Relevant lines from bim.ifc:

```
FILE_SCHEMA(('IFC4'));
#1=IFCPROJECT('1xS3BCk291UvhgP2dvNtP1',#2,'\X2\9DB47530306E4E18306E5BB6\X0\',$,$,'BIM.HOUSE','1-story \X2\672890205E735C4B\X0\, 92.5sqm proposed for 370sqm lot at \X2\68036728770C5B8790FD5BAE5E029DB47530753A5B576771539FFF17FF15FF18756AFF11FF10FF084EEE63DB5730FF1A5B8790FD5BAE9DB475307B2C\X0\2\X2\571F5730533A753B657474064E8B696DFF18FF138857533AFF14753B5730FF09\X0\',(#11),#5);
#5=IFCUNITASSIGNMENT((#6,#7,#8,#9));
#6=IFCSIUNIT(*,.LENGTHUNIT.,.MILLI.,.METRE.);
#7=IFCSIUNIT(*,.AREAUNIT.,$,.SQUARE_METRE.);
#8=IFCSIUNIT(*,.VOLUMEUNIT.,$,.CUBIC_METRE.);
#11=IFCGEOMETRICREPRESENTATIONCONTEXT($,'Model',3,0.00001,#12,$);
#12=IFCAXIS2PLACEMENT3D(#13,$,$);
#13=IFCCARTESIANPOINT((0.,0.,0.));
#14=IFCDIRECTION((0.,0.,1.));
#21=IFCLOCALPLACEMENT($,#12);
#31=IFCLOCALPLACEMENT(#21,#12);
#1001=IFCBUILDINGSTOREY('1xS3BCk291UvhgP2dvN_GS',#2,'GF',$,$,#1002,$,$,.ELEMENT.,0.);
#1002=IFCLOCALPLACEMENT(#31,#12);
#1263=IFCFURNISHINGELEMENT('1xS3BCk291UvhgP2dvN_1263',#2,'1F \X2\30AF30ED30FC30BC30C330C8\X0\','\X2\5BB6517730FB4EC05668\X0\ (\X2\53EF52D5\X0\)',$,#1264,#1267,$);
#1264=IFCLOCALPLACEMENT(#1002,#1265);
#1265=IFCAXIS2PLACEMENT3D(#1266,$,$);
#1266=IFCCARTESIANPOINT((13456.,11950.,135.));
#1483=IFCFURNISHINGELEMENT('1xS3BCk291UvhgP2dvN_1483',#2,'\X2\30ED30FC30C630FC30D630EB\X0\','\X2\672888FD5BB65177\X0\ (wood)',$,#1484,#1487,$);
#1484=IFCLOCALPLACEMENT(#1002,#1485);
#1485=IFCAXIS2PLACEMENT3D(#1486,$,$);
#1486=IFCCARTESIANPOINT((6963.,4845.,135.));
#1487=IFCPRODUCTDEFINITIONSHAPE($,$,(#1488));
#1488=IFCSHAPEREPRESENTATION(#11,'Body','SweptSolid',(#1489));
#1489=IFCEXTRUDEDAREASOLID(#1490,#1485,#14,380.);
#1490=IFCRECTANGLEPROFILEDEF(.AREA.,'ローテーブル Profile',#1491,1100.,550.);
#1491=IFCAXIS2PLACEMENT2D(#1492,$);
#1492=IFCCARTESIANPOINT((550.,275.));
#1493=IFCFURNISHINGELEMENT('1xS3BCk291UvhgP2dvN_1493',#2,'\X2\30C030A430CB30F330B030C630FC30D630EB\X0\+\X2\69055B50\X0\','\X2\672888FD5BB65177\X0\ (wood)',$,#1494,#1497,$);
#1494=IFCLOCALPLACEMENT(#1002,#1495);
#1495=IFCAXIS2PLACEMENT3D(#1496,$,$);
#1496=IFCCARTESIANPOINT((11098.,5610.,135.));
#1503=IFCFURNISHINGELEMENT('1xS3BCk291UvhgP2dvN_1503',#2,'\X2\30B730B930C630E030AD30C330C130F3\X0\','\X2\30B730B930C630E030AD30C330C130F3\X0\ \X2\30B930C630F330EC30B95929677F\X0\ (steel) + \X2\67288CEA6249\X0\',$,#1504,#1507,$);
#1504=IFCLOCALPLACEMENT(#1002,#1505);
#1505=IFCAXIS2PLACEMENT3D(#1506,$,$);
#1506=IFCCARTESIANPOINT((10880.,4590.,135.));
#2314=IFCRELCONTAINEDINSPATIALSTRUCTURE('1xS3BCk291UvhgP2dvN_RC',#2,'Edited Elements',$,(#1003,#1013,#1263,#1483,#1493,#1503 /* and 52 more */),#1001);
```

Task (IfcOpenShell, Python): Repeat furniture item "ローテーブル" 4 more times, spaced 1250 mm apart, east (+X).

```python
import numpy as np
import ifcopenshell
import ifcopenshell.api.geometry
import ifcopenshell.api.root
import ifcopenshell.util.element
import ifcopenshell.util.placement
import ifcopenshell.util.unit

model = ifcopenshell.open("bim.ifc")
unit_scale = ifcopenshell.util.unit.calculate_unit_scale(model)


def reuse_history(source, copy):
    """copy_class also copies each property set's owner history, people and application; keep the originals."""
    for rel in copy.IsDefinedBy:
        if rel.is_a("IfcRelDefinesByProperties") and (history := rel.RelatingPropertyDefinition.OwnerHistory):
            rel.RelatingPropertyDefinition.OwnerHistory = source.OwnerHistory
            ifcopenshell.util.element.remove_deep2(model, history)


source = model.by_id(1483)
base = ifcopenshell.util.placement.get_local_placement(source.ObjectPlacement)
step = np.array([1.0, 0.0, 0.0]) * 1.25 / unit_scale

for i in range(1, 5):
    copy = ifcopenshell.api.root.copy_class(model, product=source)
    copy.Representation = ifcopenshell.util.element.copy_deep(
        model, source.Representation, exclude=["IfcGeometricRepresentationContext", "IfcRepresentationMap"]
    )
    reuse_history(source, copy)
    matrix = base.copy()
    matrix[:3, 3] += i * step
    print("added at", matrix[:3, 3].round(3) + 0.0)
    ifcopenshell.api.geometry.edit_object_placement(model, product=copy, matrix=matrix, is_si=False)

model.write("bim_v2.ifc")
```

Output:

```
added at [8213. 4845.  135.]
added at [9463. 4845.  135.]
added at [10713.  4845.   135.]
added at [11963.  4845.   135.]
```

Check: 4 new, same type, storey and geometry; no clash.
